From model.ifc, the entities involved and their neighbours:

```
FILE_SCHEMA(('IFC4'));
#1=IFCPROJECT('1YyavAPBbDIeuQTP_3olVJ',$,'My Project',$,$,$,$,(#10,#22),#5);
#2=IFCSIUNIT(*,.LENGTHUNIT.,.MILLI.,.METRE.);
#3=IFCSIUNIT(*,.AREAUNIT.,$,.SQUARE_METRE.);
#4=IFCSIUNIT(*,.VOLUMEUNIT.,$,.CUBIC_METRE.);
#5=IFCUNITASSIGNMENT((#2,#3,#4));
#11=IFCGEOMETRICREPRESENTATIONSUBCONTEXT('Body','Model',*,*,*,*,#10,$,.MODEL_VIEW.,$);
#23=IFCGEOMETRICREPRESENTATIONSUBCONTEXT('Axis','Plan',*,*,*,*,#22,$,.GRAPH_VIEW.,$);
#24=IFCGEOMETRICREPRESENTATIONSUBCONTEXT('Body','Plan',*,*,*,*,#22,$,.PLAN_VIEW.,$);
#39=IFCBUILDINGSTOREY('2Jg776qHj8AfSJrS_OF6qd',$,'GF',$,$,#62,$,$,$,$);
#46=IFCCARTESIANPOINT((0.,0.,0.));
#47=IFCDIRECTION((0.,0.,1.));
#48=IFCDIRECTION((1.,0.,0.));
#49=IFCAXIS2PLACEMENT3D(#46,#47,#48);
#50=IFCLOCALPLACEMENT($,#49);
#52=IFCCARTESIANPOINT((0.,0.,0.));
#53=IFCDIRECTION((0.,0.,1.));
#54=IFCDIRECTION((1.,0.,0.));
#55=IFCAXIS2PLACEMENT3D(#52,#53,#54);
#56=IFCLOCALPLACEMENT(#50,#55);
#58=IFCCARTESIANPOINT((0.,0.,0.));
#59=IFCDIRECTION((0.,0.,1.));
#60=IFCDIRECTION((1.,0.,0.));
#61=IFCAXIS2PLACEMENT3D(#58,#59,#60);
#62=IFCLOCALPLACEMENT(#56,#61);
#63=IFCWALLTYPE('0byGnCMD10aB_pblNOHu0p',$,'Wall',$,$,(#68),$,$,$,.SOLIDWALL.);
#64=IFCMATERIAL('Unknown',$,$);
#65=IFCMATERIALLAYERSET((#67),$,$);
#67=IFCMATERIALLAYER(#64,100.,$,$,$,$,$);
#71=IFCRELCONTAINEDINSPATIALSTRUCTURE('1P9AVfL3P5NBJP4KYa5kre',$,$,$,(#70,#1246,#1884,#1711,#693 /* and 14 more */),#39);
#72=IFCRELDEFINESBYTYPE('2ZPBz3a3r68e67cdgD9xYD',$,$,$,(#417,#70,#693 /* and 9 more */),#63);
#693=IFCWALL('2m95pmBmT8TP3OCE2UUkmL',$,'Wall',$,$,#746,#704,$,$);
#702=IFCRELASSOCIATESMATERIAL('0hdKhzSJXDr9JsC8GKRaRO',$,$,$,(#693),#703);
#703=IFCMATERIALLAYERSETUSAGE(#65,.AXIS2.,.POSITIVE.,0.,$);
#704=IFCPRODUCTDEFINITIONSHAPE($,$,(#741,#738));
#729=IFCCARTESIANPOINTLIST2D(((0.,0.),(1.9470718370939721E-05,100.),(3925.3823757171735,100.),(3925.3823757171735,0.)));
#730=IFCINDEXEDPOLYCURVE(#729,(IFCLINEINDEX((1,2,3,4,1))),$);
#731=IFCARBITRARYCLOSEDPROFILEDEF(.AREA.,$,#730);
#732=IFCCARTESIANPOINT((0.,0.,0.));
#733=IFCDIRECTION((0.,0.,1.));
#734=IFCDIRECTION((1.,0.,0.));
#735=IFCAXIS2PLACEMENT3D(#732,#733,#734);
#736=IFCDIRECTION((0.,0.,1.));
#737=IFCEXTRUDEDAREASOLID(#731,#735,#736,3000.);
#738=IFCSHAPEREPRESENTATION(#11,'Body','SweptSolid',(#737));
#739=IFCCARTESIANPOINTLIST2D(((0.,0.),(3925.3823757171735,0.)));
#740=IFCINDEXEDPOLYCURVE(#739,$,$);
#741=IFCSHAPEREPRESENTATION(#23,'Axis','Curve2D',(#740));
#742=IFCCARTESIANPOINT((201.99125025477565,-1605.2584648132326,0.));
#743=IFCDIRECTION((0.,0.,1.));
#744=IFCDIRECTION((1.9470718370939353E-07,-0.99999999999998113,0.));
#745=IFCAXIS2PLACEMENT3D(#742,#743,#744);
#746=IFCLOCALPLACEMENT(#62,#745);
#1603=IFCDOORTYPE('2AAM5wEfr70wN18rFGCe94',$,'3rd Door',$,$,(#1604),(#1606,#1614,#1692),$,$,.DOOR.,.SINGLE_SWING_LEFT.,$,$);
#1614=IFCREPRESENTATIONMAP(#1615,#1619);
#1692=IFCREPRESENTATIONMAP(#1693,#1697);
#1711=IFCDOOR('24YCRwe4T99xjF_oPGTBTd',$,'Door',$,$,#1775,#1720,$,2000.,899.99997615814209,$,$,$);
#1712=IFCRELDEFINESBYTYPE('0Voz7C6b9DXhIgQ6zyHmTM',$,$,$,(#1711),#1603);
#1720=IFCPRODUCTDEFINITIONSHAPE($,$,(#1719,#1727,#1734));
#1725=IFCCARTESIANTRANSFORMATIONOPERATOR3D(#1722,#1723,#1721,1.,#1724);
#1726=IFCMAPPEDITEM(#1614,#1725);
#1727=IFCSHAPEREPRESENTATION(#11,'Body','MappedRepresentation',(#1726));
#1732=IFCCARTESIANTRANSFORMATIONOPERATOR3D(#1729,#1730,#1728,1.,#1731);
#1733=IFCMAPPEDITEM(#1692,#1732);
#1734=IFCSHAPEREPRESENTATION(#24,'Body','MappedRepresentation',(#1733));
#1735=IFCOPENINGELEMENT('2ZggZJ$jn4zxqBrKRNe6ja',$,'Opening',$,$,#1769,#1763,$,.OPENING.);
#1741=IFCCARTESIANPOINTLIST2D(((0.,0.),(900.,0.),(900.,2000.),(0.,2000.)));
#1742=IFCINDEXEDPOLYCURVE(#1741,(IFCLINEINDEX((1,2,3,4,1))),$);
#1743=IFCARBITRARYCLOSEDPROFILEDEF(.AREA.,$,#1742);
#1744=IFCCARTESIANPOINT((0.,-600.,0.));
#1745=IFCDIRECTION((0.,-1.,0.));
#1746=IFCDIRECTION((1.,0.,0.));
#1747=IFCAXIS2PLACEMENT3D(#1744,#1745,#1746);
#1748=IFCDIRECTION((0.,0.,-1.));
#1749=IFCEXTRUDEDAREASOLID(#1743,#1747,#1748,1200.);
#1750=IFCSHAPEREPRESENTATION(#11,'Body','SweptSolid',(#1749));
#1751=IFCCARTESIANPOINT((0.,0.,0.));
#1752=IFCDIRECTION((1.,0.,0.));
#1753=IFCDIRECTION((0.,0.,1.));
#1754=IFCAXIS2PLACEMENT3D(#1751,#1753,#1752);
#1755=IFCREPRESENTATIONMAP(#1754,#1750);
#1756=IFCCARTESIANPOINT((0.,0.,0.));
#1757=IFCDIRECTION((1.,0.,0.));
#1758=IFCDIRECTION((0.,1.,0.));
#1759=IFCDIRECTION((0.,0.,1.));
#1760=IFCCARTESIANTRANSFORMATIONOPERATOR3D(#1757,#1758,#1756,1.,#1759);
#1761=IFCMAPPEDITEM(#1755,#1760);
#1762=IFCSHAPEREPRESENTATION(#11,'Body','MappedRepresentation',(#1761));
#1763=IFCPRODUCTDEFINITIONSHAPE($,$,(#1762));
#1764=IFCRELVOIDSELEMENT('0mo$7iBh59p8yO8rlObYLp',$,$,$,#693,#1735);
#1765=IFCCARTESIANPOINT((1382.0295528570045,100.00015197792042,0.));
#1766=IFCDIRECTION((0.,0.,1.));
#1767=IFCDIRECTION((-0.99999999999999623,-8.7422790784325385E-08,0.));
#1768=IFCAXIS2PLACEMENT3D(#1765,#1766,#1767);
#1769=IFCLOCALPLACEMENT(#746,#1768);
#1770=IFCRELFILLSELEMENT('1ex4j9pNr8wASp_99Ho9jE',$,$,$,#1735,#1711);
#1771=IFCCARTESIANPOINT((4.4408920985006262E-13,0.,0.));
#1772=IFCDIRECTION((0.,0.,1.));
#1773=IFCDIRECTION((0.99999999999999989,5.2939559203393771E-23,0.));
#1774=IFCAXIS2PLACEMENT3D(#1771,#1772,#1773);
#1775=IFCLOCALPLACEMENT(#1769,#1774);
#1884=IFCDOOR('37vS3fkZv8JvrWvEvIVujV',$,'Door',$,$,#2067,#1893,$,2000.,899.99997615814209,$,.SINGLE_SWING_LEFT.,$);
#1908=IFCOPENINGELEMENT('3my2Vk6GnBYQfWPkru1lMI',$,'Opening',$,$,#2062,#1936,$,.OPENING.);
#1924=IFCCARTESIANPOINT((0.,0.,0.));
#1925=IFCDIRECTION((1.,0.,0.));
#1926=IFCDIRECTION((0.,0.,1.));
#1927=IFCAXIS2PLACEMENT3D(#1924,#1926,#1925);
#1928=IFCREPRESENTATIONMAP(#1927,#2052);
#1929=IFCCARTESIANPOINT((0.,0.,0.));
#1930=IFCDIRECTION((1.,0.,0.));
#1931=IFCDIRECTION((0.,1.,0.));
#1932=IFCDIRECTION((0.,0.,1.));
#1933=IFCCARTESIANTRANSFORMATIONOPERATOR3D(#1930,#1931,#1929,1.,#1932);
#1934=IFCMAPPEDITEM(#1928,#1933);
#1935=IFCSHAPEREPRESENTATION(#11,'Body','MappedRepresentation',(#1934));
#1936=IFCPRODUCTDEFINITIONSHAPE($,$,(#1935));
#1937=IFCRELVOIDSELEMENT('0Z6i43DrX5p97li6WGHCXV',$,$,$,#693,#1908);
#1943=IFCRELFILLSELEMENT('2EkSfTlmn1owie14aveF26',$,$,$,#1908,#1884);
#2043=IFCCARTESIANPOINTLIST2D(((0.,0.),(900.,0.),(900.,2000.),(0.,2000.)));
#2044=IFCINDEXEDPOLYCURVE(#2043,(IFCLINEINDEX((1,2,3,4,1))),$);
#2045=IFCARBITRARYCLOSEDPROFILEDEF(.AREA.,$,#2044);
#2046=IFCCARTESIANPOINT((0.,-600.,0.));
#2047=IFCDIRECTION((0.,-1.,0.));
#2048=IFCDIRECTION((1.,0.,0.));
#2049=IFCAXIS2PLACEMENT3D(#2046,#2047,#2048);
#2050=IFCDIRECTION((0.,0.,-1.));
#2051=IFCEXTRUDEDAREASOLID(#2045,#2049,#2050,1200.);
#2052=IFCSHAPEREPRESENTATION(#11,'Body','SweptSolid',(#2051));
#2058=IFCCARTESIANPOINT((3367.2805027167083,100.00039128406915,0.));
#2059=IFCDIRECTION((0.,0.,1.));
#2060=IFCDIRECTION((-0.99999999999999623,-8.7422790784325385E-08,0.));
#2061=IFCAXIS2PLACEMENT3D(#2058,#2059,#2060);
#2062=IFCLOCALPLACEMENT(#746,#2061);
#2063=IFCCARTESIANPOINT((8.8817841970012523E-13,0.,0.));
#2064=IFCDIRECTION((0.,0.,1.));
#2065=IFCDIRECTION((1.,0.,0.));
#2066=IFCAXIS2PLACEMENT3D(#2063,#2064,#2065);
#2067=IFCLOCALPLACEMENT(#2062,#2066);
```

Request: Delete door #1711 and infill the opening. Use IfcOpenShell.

```python
import ifcopenshell
import ifcopenshell.api.feature
import ifcopenshell.api.root
import ifcopenshell.geom
import ifcopenshell.util.shape

model = ifcopenshell.open("model.ifc")
settings = ifcopenshell.geom.settings()


def volume(element):
    """Net volume in cubic metres, openings subtracted."""
    shape = ifcopenshell.geom.create_shape(settings, element)
    return ifcopenshell.util.shape.get_volume(shape.geometry)


door = model.by_guid("24YCRwe4T99xjF_oPGTBTd")
opening = door.FillsVoids[0].RelatingOpeningElement
wall = opening.VoidsElements[0].RelatingBuildingElement
before = volume(wall)

ifcopenshell.api.root.remove_product(model, product=door)
ifcopenshell.api.feature.remove_feature(model, feature=opening)

after = volume(wall)

print(f"wall volume {before:.3f} -> {after:.3f} m3")

model.write("model_updated.ifc")
```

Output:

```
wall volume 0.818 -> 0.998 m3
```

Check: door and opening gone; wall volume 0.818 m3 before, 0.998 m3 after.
